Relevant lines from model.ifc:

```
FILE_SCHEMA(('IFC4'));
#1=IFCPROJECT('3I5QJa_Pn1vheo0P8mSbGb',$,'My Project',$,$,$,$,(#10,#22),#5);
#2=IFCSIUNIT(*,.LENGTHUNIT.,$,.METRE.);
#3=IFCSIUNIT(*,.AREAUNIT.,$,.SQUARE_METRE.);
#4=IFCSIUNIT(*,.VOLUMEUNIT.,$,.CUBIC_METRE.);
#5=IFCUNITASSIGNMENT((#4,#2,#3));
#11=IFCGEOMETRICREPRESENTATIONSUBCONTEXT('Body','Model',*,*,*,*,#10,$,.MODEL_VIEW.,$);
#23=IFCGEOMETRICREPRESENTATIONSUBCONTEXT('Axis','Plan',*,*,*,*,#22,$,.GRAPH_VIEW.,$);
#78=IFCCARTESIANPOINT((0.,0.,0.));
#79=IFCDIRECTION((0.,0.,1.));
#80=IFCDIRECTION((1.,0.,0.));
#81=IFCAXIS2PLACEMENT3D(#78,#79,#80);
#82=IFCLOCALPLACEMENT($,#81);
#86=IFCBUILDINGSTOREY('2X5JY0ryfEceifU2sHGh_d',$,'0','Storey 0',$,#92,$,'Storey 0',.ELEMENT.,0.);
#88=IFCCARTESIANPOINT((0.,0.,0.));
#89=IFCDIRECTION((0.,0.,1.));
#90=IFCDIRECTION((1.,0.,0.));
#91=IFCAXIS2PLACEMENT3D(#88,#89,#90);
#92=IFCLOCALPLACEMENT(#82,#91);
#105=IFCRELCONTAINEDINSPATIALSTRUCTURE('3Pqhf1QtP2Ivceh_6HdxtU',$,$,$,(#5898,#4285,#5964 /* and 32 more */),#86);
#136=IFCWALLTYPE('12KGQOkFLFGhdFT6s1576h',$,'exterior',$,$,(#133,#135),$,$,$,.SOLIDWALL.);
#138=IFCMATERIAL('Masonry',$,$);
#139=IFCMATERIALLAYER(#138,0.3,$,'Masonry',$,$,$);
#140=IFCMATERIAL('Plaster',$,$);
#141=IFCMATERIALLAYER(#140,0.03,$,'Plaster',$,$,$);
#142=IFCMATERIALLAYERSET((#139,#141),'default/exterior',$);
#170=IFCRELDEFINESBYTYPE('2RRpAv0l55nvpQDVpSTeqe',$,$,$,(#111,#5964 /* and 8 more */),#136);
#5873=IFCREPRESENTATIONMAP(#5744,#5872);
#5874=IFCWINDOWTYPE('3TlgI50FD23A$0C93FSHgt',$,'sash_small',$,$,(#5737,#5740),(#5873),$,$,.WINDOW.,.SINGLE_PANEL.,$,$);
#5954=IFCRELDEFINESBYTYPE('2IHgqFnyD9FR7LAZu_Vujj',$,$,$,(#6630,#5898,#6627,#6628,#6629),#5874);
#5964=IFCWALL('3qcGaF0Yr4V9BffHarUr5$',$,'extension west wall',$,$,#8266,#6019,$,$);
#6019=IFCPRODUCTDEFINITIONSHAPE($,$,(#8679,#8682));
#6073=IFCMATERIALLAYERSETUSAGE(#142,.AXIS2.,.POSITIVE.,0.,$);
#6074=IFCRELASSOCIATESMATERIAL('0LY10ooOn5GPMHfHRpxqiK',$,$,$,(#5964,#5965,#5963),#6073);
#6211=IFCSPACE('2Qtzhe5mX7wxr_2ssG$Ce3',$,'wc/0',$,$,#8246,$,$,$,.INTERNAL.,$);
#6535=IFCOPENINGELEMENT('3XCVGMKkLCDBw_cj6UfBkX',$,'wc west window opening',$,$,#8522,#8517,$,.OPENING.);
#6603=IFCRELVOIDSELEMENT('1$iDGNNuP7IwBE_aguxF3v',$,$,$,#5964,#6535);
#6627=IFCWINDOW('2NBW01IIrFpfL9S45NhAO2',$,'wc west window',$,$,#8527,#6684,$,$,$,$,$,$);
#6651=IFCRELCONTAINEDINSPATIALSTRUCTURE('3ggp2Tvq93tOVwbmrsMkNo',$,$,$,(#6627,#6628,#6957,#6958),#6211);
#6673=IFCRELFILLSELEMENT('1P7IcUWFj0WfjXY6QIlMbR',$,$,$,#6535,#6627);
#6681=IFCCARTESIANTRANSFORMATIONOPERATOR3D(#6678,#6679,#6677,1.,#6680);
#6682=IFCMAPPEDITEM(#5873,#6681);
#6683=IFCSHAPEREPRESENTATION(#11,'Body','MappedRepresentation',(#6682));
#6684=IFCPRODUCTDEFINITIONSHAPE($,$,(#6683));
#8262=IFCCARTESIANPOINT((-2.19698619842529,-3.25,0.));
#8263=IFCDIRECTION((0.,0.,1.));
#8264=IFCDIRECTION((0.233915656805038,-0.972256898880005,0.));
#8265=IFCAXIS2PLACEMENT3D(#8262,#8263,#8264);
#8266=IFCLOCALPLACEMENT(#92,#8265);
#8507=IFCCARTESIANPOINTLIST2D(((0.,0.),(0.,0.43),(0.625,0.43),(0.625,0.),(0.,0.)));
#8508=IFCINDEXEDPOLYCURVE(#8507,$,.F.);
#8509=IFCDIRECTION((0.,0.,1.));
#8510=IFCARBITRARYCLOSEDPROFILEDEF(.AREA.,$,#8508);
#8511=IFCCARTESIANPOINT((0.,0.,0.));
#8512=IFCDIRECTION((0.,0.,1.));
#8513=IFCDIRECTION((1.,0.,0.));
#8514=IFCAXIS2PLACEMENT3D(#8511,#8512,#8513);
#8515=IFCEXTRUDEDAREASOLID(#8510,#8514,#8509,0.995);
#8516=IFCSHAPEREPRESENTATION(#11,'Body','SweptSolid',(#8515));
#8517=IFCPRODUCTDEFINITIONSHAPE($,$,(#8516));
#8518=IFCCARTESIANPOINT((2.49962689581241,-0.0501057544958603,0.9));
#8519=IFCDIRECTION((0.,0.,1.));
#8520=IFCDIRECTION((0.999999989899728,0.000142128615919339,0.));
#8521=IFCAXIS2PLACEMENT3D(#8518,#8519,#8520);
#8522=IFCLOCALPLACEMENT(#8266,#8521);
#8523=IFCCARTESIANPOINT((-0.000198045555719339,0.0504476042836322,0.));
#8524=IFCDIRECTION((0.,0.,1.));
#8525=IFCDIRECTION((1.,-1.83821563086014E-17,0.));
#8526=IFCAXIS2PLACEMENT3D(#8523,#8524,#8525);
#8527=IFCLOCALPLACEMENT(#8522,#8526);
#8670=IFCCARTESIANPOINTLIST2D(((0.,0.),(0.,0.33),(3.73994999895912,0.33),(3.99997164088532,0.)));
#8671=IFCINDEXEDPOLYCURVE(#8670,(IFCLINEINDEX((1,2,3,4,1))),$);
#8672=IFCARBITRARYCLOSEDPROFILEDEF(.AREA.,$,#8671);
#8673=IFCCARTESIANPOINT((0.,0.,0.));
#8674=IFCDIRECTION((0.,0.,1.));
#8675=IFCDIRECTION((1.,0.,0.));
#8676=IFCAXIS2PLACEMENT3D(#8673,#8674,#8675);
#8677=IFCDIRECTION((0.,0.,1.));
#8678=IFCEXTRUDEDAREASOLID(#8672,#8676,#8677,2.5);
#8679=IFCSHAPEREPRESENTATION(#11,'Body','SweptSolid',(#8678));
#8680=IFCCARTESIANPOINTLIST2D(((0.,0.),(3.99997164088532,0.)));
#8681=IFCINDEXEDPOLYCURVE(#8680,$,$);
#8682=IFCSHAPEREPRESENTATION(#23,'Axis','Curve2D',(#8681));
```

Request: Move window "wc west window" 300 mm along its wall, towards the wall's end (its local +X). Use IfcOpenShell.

```python
import ifcopenshell
import ifcopenshell.api.geometry
import ifcopenshell.util.placement
import ifcopenshell.util.unit

model = ifcopenshell.open("model.ifc")
unit_scale = ifcopenshell.util.unit.calculate_unit_scale(model)

window = model.by_id(6627)
opening = window.FillsVoids[0].RelatingOpeningElement
wall = opening.VoidsElements[0].RelatingBuildingElement

wall_matrix = ifcopenshell.util.placement.get_local_placement(wall.ObjectPlacement)
shift = wall_matrix[:3, 0] * 0.3 / unit_scale
before = ifcopenshell.util.placement.get_local_placement(window.ObjectPlacement)[:3, 3].copy()

# The window is placed relative to its opening, so it follows when the opening moves.
matrix = ifcopenshell.util.placement.get_local_placement(opening.ObjectPlacement)
matrix[:3, 3] += shift
ifcopenshell.api.geometry.edit_object_placement(
    model, product=opening, matrix=matrix, is_si=False, should_transform_children=True
)

after = ifcopenshell.util.placement.get_local_placement(window.ObjectPlacement)[:3, 3]
print("window moved by", (after - before).round(3) + 0.0)

model.write("model_edited.ifc")
```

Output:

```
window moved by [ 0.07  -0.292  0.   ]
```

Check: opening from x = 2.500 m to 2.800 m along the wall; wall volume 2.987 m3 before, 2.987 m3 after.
